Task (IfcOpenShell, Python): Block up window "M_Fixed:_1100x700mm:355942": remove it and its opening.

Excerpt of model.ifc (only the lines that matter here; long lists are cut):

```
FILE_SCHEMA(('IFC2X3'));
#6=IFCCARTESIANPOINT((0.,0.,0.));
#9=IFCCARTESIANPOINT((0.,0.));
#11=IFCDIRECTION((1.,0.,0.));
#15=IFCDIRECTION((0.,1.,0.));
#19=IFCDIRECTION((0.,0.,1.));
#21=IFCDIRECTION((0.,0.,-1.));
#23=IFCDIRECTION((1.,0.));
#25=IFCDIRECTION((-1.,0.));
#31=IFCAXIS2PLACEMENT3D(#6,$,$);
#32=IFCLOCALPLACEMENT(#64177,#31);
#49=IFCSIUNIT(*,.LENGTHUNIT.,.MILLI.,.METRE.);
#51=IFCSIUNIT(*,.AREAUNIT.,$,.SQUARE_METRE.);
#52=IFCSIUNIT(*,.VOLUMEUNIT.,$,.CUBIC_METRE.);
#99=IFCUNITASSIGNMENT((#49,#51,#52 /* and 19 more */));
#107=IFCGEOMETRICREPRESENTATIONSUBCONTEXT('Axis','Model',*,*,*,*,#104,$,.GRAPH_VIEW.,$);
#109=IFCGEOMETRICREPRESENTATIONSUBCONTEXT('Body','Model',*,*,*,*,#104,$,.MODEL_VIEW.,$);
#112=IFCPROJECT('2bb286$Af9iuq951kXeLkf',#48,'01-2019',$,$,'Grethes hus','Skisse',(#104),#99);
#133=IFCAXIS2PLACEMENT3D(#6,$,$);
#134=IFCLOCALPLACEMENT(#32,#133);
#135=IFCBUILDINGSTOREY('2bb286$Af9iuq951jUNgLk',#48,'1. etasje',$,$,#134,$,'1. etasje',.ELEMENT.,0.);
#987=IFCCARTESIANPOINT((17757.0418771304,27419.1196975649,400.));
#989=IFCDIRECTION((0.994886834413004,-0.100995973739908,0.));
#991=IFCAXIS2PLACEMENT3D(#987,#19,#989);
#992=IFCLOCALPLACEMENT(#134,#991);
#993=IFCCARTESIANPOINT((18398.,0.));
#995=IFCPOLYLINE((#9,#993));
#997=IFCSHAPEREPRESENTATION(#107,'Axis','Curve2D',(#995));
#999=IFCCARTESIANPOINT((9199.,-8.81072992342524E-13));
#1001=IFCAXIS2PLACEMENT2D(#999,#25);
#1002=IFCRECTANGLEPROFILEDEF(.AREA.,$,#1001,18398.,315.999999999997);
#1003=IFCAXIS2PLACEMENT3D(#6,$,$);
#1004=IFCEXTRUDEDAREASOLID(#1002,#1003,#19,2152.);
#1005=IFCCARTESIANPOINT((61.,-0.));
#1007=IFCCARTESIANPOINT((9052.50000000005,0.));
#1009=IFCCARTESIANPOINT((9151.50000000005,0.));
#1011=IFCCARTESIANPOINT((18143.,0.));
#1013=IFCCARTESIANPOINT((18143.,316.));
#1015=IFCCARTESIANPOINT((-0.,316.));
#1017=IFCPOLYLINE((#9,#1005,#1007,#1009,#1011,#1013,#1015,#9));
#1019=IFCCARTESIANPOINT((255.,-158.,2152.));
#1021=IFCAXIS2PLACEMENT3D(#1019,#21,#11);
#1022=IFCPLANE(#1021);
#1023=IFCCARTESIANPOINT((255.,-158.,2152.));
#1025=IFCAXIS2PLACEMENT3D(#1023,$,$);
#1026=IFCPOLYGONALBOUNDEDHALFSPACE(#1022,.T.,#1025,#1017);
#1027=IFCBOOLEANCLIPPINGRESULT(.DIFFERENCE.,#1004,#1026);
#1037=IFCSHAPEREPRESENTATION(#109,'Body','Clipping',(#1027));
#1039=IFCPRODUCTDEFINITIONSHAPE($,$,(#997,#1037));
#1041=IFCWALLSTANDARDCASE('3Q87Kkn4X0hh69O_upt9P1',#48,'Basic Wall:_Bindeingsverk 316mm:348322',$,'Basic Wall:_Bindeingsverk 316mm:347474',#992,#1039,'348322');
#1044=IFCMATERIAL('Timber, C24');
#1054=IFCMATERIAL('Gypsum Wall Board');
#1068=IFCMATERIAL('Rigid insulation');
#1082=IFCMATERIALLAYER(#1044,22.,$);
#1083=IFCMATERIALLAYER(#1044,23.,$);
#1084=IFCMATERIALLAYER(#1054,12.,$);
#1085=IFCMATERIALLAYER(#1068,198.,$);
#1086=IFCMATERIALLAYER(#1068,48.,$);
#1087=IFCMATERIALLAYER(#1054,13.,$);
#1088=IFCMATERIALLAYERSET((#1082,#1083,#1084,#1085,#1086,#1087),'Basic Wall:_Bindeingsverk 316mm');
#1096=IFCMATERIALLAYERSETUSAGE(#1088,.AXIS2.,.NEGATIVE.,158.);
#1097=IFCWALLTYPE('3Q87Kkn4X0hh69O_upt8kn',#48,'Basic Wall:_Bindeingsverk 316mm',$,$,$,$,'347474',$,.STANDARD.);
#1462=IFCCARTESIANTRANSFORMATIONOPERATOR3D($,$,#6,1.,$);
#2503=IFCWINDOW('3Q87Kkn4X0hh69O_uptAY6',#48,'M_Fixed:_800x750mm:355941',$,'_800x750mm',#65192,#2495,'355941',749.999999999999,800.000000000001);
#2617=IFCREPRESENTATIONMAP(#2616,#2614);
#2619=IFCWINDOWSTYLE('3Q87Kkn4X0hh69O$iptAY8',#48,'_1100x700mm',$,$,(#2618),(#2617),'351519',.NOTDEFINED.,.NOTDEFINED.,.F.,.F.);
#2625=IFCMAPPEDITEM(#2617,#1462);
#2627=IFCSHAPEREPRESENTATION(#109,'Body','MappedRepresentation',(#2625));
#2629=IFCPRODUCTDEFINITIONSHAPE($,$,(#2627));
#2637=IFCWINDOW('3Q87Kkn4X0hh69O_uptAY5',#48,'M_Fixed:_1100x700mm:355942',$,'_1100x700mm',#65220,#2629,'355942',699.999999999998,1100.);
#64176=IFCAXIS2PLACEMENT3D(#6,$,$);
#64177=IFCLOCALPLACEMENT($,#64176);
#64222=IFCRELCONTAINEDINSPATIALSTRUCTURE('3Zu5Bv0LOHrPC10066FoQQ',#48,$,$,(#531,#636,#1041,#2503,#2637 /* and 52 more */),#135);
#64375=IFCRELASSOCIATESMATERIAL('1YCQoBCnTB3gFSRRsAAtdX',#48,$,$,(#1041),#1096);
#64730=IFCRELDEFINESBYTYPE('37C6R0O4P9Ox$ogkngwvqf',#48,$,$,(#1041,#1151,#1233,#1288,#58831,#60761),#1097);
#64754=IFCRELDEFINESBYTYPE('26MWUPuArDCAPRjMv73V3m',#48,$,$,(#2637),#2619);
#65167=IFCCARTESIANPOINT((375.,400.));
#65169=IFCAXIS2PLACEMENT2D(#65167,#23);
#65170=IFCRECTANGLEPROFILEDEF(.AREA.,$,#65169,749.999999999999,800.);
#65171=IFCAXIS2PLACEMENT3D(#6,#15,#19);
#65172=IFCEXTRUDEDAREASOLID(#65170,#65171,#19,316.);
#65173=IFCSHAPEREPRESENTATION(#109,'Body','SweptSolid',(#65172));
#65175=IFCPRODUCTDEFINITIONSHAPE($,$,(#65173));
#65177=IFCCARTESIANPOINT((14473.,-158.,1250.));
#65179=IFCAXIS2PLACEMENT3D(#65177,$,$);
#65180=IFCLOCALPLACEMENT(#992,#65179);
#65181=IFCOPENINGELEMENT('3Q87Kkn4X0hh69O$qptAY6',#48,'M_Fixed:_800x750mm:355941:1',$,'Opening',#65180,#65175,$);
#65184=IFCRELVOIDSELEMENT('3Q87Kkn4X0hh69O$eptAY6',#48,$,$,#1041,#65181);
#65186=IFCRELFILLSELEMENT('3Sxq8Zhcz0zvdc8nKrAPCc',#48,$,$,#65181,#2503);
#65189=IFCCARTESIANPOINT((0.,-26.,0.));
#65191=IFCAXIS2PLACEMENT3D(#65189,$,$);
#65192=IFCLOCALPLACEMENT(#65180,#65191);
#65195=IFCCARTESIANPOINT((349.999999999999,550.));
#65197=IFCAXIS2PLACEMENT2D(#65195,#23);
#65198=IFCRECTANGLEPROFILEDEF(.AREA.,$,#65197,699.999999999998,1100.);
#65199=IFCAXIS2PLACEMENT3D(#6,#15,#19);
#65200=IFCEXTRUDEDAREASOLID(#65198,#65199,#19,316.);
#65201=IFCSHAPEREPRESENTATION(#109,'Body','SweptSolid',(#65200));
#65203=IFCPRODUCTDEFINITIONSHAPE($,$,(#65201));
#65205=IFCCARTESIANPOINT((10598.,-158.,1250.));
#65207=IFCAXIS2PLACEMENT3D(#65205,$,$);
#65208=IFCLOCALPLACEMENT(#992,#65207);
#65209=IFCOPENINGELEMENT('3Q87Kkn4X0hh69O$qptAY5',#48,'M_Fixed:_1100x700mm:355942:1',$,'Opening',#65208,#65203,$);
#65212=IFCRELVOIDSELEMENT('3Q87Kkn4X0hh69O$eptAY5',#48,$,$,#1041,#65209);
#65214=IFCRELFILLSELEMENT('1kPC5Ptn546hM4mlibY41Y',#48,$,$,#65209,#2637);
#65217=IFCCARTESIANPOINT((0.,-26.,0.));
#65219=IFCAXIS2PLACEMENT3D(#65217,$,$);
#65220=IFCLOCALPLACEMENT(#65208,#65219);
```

```python
import ifcopenshell
import ifcopenshell.api.feature
import ifcopenshell.api.root
import ifcopenshell.geom
import ifcopenshell.util.shape

model = ifcopenshell.open("model.ifc")
settings = ifcopenshell.geom.settings()


def volume(element):
    """Net volume in cubic metres, openings subtracted."""
    shape = ifcopenshell.geom.create_shape(settings, element)
    return ifcopenshell.util.shape.get_volume(shape.geometry)


window = model.by_id(2637)
opening = window.FillsVoids[0].RelatingOpeningElement
wall = opening.VoidsElements[0].RelatingBuildingElement
before = volume(wall)

ifcopenshell.api.root.remove_product(model, product=window)
ifcopenshell.api.feature.remove_feature(model, feature=opening)

after = volume(wall)

print(f"wall volume {before:.3f} -> {after:.3f} m3")

model.write("model_updated.ifc")
```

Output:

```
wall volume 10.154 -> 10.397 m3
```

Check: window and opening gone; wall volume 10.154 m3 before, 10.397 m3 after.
